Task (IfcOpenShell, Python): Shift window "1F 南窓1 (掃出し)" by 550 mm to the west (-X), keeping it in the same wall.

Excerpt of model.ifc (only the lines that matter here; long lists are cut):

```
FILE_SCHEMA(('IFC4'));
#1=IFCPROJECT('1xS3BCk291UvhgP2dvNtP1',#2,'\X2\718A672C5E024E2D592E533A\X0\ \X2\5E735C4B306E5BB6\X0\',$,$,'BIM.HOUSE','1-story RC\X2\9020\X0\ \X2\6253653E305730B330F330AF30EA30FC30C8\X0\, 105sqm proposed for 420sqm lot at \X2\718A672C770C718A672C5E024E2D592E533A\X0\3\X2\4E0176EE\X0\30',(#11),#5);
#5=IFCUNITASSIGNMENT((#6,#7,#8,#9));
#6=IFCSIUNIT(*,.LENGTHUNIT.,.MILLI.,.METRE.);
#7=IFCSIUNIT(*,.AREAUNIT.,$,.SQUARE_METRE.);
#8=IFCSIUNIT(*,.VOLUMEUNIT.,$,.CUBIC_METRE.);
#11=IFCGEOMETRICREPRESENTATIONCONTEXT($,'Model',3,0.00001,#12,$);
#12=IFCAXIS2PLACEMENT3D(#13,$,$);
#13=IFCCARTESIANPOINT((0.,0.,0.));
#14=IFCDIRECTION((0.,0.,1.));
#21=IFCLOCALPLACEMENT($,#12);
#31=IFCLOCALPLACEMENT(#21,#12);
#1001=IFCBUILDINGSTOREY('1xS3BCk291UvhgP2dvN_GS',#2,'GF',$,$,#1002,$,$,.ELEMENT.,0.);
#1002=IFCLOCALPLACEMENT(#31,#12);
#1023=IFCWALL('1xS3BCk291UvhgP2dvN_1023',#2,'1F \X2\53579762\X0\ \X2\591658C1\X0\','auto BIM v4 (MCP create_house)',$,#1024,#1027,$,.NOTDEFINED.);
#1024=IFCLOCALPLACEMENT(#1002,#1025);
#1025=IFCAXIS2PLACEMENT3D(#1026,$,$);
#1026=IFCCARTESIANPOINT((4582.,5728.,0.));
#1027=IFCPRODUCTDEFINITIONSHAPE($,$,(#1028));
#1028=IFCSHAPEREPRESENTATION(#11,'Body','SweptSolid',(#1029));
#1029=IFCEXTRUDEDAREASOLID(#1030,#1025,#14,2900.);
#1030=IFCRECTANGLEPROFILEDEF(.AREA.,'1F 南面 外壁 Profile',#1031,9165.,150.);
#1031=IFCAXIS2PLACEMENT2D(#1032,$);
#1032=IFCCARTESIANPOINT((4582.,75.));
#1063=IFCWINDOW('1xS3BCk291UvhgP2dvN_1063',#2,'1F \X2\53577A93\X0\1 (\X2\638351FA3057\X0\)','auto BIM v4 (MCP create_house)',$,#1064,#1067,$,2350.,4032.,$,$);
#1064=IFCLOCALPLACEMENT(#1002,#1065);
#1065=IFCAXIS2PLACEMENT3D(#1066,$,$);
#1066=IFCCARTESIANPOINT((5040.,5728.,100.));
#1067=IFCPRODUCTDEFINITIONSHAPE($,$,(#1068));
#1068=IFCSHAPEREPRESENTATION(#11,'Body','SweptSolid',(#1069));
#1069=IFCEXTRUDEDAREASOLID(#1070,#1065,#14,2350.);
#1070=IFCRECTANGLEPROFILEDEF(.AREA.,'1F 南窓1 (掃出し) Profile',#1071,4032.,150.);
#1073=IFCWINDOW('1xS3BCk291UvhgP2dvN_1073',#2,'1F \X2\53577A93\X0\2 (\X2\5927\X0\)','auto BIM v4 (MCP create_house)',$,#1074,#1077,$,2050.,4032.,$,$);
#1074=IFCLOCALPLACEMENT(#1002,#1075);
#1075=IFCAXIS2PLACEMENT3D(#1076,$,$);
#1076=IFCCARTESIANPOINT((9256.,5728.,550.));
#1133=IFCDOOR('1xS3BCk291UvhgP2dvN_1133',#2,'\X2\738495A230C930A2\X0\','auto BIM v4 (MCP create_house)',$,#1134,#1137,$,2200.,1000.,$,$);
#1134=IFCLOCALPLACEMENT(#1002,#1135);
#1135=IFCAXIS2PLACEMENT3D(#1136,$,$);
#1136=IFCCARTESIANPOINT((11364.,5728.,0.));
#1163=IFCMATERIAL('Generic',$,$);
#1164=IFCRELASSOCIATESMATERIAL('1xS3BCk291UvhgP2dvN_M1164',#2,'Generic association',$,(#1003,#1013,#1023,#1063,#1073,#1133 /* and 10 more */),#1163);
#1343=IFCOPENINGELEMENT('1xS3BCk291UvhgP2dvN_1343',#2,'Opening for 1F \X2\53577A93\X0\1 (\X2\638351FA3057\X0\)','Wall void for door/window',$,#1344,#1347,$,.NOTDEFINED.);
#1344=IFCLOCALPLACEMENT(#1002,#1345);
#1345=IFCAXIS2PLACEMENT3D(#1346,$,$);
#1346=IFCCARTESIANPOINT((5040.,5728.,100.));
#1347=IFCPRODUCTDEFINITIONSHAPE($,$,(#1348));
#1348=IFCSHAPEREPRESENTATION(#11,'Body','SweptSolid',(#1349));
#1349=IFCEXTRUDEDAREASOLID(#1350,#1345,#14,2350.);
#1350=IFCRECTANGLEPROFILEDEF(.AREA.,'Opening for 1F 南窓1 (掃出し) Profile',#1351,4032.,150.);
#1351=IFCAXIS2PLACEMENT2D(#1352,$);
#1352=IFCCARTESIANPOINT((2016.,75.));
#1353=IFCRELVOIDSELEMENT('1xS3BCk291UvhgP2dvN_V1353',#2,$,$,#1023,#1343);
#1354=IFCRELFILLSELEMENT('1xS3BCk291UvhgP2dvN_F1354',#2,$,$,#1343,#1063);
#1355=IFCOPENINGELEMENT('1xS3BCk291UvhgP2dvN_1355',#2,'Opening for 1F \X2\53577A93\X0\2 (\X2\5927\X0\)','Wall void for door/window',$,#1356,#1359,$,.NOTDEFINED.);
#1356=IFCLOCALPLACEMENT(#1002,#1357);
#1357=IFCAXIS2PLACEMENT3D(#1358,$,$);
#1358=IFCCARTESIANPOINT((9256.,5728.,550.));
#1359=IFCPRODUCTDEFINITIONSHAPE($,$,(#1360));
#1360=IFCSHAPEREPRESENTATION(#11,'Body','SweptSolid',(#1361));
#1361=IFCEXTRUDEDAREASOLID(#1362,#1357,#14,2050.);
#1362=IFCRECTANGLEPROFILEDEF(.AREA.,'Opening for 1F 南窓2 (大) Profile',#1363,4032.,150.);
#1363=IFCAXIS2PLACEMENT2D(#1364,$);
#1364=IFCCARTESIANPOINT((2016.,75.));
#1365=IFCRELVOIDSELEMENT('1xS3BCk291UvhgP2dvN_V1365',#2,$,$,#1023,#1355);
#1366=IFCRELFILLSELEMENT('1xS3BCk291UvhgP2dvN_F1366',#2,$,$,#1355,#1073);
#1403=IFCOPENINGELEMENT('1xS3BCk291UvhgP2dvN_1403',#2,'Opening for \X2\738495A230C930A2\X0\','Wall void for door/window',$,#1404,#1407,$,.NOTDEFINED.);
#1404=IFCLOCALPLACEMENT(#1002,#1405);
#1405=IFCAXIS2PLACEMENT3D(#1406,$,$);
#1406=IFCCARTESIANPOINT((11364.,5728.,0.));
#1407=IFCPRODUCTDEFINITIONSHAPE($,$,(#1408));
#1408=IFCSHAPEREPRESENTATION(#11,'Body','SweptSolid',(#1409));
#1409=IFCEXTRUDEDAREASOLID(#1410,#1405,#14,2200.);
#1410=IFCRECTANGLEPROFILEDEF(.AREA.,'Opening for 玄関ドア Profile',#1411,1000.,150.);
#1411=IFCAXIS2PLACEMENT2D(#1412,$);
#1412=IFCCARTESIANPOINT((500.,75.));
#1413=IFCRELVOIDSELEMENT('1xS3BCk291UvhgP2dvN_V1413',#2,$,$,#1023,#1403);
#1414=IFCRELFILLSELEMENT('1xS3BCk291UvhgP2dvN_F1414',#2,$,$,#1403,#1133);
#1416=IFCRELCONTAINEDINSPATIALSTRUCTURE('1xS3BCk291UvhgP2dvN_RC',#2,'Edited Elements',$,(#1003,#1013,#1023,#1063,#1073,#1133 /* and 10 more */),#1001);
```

```python
import ifcopenshell
import ifcopenshell.api.geometry
import ifcopenshell.util.placement
import ifcopenshell.util.unit

model = ifcopenshell.open("model.ifc")
unit_scale = ifcopenshell.util.unit.calculate_unit_scale(model)

window = model.by_id(1063)
opening = window.FillsVoids[0].RelatingOpeningElement
wall = opening.VoidsElements[0].RelatingBuildingElement

wall_matrix = ifcopenshell.util.placement.get_local_placement(wall.ObjectPlacement)
shift = wall_matrix[:3, 0] * -0.55 / unit_scale
before = ifcopenshell.util.placement.get_local_placement(window.ObjectPlacement)[:3, 3].copy()

# The window is not placed relative to its opening, so move both.
for product in (opening, window):
    matrix = ifcopenshell.util.placement.get_local_placement(product.ObjectPlacement)
    matrix[:3, 3] += shift
    ifcopenshell.api.geometry.edit_object_placement(model, product=product, matrix=matrix, is_si=False)

after = ifcopenshell.util.placement.get_local_placement(window.ObjectPlacement)[:3, 3]
print("window moved by", (after - before).round(3) + 0.0)

model.write("model_v2.ifc")
```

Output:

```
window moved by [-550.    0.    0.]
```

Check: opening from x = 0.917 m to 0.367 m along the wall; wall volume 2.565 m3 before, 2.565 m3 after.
